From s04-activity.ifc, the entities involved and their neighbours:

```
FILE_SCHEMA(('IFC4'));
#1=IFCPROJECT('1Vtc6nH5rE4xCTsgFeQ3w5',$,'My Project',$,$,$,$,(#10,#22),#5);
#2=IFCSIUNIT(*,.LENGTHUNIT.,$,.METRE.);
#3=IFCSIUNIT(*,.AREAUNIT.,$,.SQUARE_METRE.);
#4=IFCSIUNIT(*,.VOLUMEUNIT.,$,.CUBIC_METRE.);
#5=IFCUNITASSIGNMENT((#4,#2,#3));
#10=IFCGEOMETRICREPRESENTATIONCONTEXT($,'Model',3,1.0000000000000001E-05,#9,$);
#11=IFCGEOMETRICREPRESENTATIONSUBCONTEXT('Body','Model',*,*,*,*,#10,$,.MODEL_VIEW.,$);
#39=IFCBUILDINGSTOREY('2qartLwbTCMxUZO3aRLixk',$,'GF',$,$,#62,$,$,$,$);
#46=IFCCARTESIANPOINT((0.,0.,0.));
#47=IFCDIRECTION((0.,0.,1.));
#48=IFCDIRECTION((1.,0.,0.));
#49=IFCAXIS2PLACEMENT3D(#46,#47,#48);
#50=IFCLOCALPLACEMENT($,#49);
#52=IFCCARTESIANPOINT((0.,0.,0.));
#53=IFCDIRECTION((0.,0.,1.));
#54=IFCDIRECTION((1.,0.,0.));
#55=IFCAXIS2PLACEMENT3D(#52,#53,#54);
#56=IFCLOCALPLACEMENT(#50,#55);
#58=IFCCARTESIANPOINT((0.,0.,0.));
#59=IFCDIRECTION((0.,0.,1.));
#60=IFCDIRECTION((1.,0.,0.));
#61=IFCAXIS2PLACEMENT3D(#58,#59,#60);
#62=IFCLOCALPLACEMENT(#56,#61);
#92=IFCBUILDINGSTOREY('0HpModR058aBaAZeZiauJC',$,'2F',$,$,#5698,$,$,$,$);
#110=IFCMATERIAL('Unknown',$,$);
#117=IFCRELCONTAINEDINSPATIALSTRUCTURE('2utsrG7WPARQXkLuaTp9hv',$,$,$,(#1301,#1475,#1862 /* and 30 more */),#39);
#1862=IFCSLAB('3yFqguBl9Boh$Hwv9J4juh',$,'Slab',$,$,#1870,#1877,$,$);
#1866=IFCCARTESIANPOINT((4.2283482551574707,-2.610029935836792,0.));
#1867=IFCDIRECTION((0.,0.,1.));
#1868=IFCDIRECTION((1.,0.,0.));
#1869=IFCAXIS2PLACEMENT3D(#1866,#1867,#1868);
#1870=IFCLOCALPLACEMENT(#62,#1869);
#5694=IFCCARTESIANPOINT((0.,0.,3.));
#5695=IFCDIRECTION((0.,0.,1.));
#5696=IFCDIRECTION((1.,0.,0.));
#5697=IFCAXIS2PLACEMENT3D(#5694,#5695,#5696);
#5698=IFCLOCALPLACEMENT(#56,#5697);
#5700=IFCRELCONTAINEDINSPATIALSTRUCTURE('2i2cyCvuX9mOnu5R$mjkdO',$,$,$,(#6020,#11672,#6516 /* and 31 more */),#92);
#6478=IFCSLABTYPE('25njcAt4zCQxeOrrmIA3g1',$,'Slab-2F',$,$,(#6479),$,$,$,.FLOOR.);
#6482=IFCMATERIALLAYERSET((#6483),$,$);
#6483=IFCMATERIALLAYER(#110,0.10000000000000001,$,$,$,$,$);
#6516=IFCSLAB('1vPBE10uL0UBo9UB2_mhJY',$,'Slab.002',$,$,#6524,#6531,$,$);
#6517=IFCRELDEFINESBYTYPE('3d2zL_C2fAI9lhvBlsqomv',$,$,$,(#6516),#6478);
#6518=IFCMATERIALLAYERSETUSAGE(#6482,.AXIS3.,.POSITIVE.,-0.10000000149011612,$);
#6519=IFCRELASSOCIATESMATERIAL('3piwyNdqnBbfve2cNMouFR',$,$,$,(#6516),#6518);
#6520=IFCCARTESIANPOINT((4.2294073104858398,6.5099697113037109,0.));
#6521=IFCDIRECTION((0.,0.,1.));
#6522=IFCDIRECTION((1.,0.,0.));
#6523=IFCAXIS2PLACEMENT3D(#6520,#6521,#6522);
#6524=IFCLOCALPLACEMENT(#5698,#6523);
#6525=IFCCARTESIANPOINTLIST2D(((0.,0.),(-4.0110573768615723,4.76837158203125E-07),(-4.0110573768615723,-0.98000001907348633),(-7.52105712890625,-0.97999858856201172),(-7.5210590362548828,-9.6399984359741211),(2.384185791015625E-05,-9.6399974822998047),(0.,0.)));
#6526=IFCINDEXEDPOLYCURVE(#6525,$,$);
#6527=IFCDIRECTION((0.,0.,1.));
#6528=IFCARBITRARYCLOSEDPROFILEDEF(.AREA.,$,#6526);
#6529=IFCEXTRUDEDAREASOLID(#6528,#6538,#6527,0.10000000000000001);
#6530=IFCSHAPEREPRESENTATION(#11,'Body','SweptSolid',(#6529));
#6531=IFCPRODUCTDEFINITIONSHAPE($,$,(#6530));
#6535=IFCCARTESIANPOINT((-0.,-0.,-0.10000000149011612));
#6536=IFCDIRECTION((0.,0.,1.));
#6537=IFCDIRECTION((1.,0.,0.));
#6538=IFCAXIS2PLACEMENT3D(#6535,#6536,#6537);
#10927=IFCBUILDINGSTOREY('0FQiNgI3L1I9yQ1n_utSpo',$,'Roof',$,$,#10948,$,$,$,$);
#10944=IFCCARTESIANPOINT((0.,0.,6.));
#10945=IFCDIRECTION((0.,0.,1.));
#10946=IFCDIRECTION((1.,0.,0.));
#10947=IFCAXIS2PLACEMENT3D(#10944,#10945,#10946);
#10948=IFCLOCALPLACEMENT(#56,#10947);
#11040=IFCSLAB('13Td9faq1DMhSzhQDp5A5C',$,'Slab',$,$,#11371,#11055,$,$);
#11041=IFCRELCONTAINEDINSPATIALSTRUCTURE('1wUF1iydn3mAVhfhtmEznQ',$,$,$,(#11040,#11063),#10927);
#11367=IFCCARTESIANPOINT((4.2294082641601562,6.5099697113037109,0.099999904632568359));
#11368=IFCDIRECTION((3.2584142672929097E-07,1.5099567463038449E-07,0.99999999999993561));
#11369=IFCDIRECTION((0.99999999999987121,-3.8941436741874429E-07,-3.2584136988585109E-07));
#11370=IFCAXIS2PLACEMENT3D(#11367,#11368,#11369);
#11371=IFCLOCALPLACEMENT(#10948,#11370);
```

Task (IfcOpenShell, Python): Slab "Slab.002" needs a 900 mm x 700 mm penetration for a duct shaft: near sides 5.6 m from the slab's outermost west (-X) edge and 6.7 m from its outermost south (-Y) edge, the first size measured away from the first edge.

```python
import numpy as np
import ifcopenshell
import ifcopenshell.api.feature
import ifcopenshell.api.geometry
import ifcopenshell.api.root
import ifcopenshell.geom
import ifcopenshell.util.placement
import ifcopenshell.util.representation
import ifcopenshell.util.shape
import ifcopenshell.util.unit

model = ifcopenshell.open("s04-activity.ifc")
unit_scale = ifcopenshell.util.unit.calculate_unit_scale(model)
settings = ifcopenshell.geom.settings()


def volume(element):
    """Net volume in cubic metres, openings subtracted."""
    shape = ifcopenshell.geom.create_shape(settings, element)
    return ifcopenshell.util.shape.get_volume(shape.geometry)


slab = model.by_guid("1vPBE10uL0UBo9UB2_mhJY")
before = volume(slab)

# Extent in the slab's own axes, in metres. The edges named are its -X and -Y sides.
slab_shape = ifcopenshell.geom.create_shape(settings, slab)
vertices = ifcopenshell.util.shape.get_vertices(slab_shape.geometry)
x_min, y_min, bottom = vertices.min(axis=0)
top = vertices[:, 2].max()

opening = ifcopenshell.api.root.create_entity(model, ifc_class="IfcOpeningElement", name="Duct shaft opening", predefined_type="OPENING")
context = ifcopenshell.util.representation.get_context(model, "Model", "Body", "MODEL_VIEW")
width, depth = 0.9, 0.7
outline = [(0.0, 0.0), (width, 0.0), (width, depth), (0.0, depth), (0.0, 0.0)]
# Overshoot both faces by 50 mm so the cut is clean.
shape = ifcopenshell.api.geometry.add_slab_representation(
    model, context=context, depth=top - bottom + 0.1, polyline=outline
)
ifcopenshell.api.geometry.assign_representation(model, product=opening, representation=shape)

matrix = ifcopenshell.util.placement.get_local_placement(slab.ObjectPlacement)
matrix[:, 3] = matrix @ np.append(np.array([x_min + 5.6, y_min + 6.7, bottom - 0.05]) / unit_scale, 1.0)
ifcopenshell.api.geometry.edit_object_placement(model, product=opening, matrix=matrix, is_si=False)
ifcopenshell.api.feature.add_feature(model, feature=opening, element=slab)

after = volume(slab)

print(f"slab volume {before:.3f} -> {after:.3f} m3")

model.write("s04-activity_edited.ifc")
```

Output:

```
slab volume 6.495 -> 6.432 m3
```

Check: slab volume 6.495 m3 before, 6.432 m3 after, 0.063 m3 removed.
